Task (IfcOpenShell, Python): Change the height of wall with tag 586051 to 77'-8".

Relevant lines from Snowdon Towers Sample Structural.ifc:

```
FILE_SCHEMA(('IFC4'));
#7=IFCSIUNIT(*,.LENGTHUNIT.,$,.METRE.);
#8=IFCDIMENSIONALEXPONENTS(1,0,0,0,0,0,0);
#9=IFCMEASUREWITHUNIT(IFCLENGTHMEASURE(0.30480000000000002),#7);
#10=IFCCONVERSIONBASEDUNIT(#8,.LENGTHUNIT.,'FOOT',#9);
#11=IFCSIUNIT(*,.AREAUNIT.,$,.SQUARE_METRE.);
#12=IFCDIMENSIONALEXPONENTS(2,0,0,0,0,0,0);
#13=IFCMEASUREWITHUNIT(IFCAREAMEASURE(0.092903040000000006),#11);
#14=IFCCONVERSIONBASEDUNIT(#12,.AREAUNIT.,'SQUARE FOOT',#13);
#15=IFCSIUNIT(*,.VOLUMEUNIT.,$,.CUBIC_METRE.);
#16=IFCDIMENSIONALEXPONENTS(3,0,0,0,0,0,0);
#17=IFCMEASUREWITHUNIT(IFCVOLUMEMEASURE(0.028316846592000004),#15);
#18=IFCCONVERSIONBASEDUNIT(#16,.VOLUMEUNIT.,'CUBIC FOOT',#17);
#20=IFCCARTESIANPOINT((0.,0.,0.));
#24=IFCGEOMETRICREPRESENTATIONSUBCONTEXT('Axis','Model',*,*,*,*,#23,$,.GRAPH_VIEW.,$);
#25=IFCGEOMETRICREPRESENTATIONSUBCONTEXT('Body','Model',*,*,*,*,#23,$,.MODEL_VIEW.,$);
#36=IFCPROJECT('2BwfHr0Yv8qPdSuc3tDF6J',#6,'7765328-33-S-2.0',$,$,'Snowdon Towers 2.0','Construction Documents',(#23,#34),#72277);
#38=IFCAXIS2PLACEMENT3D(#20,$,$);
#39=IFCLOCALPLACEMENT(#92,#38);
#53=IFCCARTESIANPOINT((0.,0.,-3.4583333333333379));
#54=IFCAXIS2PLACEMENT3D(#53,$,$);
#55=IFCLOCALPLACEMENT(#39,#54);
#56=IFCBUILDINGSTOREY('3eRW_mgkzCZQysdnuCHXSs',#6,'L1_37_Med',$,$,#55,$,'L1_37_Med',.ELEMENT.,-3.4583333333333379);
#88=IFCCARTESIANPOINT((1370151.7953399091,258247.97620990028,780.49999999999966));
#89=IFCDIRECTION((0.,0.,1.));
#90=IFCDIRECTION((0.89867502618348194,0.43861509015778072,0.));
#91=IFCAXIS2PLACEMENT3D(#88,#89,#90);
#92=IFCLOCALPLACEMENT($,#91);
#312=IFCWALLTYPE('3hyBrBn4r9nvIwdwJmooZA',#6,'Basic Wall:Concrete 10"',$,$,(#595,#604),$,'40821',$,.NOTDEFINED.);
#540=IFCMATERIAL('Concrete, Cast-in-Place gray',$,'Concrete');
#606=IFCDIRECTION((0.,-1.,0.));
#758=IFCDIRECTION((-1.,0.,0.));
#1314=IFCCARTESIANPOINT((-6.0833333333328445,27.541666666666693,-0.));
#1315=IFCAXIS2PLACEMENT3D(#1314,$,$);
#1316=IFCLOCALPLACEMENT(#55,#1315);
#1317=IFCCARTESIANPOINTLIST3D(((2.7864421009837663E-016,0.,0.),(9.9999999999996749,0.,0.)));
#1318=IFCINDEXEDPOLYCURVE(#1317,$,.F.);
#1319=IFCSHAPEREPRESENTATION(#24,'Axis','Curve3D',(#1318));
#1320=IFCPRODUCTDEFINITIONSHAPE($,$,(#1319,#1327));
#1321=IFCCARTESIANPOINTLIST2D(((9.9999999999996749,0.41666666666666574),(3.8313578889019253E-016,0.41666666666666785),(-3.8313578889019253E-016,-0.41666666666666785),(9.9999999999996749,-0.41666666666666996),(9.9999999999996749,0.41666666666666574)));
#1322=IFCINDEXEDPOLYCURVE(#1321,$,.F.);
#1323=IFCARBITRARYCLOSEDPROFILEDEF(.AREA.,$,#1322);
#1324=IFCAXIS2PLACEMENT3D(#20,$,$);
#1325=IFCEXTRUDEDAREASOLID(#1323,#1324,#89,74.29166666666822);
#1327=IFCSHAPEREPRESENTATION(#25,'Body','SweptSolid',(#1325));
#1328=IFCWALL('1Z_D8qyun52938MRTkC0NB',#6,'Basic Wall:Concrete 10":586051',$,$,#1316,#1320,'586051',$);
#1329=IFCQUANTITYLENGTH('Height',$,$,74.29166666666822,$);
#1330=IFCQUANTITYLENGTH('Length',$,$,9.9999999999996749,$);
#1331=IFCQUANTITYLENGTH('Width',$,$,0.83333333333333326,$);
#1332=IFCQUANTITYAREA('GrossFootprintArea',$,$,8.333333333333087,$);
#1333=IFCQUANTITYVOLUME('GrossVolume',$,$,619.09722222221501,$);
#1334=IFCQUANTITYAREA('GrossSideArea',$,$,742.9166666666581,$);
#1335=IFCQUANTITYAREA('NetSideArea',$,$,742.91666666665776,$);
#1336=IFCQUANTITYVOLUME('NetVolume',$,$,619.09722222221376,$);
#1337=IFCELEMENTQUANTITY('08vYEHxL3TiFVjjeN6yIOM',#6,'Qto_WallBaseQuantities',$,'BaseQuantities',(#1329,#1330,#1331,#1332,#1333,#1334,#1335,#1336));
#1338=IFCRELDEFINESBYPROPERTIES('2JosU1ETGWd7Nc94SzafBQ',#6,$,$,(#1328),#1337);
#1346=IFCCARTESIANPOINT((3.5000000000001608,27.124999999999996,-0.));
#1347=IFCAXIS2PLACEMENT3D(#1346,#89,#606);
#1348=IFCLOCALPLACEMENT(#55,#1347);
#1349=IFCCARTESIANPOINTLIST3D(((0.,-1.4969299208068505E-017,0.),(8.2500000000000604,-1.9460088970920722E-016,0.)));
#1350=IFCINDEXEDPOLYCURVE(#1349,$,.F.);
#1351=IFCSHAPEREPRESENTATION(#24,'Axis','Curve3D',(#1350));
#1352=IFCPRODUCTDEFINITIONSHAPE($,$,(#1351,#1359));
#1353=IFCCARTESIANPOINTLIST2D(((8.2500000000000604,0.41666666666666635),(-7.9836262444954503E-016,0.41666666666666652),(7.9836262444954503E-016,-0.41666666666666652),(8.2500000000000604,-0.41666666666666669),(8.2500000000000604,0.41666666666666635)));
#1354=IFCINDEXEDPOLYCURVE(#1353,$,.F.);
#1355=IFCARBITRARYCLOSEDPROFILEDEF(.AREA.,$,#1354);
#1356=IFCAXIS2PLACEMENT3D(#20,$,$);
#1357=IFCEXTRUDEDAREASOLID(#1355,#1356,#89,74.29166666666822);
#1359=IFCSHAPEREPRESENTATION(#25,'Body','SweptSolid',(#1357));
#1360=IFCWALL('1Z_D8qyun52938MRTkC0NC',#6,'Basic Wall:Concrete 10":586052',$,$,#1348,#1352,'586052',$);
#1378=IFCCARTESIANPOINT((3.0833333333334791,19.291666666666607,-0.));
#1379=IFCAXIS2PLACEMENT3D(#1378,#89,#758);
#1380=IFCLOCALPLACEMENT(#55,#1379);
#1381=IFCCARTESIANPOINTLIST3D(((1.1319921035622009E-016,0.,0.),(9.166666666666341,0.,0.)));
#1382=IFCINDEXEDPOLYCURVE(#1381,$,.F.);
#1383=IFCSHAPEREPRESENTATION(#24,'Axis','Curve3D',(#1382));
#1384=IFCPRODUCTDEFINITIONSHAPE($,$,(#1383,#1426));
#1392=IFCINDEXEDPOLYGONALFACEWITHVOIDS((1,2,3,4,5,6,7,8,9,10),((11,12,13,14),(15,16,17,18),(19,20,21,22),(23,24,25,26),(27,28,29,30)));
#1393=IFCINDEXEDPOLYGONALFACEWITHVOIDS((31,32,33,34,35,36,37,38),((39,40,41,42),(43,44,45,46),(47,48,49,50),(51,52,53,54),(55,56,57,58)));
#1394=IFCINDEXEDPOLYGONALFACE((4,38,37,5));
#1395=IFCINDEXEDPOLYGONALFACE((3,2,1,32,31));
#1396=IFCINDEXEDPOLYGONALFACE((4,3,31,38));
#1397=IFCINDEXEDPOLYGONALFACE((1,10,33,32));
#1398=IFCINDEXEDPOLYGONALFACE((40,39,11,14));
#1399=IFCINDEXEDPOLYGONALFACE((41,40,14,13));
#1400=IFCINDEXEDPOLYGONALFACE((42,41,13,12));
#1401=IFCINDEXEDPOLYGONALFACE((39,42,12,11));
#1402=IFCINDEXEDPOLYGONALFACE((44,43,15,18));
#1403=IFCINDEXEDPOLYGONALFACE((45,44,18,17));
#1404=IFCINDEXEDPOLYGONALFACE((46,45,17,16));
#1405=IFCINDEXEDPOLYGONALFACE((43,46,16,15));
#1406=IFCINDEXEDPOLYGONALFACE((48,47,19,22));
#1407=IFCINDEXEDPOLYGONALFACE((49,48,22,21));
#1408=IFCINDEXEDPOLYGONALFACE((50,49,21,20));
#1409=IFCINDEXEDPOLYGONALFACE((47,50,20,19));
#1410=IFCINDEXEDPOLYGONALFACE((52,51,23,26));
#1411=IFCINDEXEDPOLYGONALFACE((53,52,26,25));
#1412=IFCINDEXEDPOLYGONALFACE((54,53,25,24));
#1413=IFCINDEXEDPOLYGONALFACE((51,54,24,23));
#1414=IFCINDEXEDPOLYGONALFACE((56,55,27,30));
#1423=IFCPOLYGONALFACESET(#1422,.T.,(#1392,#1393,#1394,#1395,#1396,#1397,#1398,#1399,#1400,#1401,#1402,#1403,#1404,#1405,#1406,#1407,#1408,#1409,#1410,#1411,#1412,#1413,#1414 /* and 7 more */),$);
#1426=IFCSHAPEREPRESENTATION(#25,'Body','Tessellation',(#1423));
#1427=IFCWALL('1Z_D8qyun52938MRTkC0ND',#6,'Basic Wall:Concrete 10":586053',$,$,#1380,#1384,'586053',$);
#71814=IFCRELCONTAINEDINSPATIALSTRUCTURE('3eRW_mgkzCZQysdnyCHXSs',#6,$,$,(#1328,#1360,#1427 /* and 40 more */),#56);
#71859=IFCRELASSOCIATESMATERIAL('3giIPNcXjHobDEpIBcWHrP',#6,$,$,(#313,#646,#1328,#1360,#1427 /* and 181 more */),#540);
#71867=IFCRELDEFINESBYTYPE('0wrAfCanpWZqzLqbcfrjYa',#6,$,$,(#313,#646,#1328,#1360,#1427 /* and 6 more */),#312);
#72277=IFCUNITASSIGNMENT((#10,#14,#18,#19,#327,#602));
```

```python
import ifcopenshell
import ifcopenshell.api.pset
import ifcopenshell.geom
import ifcopenshell.util.element
import ifcopenshell.util.representation
import ifcopenshell.util.shape
import ifcopenshell.util.unit

model = ifcopenshell.open("Snowdon Towers Sample Structural.ifc")
unit_scale = ifcopenshell.util.unit.calculate_unit_scale(model)
area_scale = ifcopenshell.util.unit.calculate_unit_scale(model, "AREAUNIT")
volume_scale = ifcopenshell.util.unit.calculate_unit_scale(model, "VOLUMEUNIT")
settings = ifcopenshell.geom.settings()


def volume(element):
    """Net volume in cubic metres, openings subtracted."""
    shape = ifcopenshell.geom.create_shape(settings, element)
    return ifcopenshell.util.shape.get_volume(shape.geometry)


wall = model.by_guid("1Z_D8qyun52938MRTkC0NB")
before = volume(wall)

body = ifcopenshell.util.representation.get_representation(wall, "Model", "Body")
solid = body.Items[0]
old_height = solid.Depth
solid.Depth = 932 * 0.0254 / unit_scale
after = volume(wall)
thickness = 0.254  # wall thickness in metres

# Update the stored height, areas and volumes.
qto = model.by_id(ifcopenshell.util.element.get_pset(wall, "Qto_WallBaseQuantities", should_inherit=False)["id"])
ifcopenshell.api.pset.edit_qto(model, qto=qto, properties={
    "Height": solid.Depth,
    "GrossVolume": ifcopenshell.util.element.get_pset(wall, "Qto_WallBaseQuantities", "GrossVolume") * solid.Depth / old_height,
    "GrossSideArea": ifcopenshell.util.element.get_pset(wall, "Qto_WallBaseQuantities", "GrossSideArea") * solid.Depth / old_height,
    "NetSideArea": after / thickness / area_scale,
    "NetVolume": after / volume_scale,
})

print(f"height {old_height:g} -> {solid.Depth:g}, volume {before:.3f} -> {after:.3f} m3")

model.write("Snowdon Towers Sample Structural_updated.ifc")
```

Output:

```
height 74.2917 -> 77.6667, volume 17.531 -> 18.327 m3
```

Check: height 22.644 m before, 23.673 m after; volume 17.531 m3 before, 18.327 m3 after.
